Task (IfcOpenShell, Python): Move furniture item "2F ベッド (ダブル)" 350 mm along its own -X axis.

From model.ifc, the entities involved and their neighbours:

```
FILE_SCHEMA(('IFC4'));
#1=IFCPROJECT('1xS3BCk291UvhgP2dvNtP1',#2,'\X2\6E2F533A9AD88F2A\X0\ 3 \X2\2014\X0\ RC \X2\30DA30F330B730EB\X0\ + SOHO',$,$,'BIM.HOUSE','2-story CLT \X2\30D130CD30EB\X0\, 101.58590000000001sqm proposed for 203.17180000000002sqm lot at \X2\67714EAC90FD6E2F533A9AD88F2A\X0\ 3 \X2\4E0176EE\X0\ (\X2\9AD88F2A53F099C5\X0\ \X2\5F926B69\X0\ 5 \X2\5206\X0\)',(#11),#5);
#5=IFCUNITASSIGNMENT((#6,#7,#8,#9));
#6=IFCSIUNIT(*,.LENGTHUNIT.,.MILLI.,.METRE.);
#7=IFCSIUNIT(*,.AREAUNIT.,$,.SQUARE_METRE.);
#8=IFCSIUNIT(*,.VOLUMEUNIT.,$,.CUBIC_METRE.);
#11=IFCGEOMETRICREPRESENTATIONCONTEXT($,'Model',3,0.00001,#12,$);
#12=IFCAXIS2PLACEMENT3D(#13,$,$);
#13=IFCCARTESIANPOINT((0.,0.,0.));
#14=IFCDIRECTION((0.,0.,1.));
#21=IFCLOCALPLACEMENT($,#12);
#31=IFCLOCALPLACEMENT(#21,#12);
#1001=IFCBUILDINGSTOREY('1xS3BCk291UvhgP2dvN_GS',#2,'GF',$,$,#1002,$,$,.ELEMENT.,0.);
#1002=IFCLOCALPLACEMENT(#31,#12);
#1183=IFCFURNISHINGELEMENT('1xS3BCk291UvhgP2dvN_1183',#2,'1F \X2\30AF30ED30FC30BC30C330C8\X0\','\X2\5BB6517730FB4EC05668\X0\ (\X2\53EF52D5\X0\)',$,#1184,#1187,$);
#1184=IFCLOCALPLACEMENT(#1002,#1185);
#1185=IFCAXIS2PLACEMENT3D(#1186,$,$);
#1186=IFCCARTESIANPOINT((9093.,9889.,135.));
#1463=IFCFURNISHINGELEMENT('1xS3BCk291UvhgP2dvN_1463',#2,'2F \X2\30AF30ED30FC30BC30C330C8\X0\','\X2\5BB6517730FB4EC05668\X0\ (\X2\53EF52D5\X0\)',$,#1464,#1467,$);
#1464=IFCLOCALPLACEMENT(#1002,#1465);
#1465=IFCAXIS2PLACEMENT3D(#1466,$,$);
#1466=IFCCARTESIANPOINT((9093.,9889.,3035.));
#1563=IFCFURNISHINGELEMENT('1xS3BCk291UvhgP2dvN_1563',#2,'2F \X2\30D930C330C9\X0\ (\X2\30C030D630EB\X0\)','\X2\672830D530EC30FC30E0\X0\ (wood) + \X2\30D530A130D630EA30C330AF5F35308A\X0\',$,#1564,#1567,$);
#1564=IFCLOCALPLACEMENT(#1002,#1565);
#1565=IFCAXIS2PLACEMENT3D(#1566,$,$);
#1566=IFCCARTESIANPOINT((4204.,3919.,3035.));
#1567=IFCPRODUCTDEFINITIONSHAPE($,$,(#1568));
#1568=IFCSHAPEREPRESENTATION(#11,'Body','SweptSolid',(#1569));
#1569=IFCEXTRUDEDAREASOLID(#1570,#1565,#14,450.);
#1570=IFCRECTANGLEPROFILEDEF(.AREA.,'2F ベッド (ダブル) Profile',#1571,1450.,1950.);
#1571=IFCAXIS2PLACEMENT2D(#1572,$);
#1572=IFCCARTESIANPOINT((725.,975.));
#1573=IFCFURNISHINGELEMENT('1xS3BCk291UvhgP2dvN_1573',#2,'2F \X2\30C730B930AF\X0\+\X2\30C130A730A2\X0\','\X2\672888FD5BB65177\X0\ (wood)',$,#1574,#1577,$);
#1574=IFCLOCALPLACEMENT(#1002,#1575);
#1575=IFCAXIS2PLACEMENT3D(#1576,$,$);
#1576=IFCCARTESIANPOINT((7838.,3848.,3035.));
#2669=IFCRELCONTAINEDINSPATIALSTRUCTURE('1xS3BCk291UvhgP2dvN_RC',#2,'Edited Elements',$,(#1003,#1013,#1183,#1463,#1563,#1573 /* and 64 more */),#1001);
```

```python
import ifcopenshell
import ifcopenshell.api.geometry
import ifcopenshell.util.placement
import ifcopenshell.util.unit

model = ifcopenshell.open("model.ifc")
unit_scale = ifcopenshell.util.unit.calculate_unit_scale(model)

item = model.by_id(1563)
matrix = ifcopenshell.util.placement.get_local_placement(item.ObjectPlacement)
matrix[:3, 3] -= matrix[:3, 0] * 0.35 / unit_scale
ifcopenshell.api.geometry.edit_object_placement(model, product=item, matrix=matrix, is_si=False)

print(ifcopenshell.util.placement.get_local_placement(item.ObjectPlacement).round(3) + 0.0)

model.write("model_edited.ifc")
```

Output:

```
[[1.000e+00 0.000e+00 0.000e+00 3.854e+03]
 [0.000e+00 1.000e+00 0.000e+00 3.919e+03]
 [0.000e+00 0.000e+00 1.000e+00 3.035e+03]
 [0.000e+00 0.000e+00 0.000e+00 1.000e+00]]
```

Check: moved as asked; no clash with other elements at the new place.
